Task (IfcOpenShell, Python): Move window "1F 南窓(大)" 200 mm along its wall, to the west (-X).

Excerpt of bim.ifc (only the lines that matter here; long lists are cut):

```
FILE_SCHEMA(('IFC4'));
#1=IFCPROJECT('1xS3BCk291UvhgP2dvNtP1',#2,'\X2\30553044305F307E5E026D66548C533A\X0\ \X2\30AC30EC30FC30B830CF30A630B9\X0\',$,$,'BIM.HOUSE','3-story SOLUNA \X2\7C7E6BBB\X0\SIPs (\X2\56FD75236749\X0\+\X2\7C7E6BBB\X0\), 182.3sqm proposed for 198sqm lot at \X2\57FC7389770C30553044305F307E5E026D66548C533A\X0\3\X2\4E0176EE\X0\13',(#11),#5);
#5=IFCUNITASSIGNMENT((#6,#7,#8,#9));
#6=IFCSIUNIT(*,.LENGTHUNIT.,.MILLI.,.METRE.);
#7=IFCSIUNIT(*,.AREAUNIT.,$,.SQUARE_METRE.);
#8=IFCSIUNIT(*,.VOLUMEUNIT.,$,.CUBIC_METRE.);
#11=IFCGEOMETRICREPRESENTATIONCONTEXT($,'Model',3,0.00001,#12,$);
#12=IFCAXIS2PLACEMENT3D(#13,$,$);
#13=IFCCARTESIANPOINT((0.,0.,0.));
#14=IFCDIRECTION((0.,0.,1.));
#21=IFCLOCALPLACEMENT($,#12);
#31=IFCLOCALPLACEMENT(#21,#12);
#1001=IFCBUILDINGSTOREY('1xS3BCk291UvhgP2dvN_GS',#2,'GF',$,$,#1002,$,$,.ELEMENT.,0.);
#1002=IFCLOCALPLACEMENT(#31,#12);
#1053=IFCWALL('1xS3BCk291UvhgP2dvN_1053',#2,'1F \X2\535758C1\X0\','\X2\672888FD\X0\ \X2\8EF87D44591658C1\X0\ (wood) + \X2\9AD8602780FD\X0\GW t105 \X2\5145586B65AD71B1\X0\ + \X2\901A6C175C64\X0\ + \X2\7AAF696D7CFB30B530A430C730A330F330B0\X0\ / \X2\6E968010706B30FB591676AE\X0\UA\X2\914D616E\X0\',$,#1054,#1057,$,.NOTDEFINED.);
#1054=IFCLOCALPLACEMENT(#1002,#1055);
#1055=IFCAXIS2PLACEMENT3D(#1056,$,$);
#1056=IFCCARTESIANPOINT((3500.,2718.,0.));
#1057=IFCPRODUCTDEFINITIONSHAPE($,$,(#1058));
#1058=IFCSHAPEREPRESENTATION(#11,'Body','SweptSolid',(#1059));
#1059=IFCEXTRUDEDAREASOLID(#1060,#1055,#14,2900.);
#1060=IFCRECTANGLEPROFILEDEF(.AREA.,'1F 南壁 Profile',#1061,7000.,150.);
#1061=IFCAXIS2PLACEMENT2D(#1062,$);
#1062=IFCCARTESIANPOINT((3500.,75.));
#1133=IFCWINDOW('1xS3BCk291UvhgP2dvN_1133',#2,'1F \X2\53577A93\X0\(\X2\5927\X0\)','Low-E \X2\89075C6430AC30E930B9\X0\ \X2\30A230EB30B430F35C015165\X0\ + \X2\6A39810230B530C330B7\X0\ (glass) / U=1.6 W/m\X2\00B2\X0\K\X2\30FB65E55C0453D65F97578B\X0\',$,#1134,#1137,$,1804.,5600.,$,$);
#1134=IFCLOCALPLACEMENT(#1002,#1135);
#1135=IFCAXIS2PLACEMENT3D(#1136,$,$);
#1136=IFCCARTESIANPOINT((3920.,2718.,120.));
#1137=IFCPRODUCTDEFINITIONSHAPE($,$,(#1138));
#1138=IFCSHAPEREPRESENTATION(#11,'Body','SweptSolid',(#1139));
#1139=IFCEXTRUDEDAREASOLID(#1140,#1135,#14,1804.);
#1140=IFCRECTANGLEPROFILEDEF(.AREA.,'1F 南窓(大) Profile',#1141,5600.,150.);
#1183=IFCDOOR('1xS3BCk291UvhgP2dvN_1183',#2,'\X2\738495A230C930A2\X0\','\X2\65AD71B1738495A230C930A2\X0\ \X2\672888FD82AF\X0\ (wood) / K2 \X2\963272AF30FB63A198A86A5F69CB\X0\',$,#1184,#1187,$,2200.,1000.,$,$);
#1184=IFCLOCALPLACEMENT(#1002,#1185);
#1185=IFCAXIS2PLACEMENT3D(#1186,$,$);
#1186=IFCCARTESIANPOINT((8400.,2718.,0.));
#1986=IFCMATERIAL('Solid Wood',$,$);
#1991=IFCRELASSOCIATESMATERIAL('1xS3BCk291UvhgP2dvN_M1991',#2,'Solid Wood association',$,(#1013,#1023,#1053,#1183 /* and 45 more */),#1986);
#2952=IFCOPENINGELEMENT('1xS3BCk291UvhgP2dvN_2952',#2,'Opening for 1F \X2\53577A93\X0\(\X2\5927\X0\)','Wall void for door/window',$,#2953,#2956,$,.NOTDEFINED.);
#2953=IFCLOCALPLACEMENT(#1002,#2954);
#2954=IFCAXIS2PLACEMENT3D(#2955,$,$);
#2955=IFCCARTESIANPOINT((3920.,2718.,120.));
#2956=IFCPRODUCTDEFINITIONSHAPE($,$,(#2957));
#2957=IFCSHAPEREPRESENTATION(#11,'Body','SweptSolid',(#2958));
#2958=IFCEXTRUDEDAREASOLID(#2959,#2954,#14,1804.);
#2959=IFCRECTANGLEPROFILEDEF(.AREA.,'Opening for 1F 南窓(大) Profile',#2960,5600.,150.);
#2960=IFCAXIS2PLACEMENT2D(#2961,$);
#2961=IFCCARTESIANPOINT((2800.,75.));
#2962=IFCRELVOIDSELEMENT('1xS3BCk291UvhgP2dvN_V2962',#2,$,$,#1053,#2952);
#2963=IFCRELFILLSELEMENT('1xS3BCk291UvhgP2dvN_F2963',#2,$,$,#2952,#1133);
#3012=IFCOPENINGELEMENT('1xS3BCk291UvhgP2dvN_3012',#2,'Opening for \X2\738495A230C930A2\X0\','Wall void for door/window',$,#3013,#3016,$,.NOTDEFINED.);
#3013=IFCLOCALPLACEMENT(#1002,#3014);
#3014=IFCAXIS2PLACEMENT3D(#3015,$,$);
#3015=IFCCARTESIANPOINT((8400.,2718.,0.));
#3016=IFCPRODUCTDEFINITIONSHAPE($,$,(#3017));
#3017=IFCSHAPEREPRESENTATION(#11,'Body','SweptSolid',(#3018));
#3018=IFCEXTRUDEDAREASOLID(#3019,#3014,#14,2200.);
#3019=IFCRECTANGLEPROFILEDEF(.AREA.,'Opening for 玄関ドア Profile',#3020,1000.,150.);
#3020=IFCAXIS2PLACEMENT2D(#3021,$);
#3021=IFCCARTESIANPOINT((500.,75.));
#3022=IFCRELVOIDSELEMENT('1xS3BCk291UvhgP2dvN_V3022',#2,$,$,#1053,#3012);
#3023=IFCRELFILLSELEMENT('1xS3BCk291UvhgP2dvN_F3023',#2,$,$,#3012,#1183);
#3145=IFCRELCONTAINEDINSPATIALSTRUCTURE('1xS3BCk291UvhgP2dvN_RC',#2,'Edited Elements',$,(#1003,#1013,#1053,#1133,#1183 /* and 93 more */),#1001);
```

```python
import ifcopenshell
import ifcopenshell.api.geometry
import ifcopenshell.util.placement

model = ifcopenshell.open("bim.ifc")

window = model.by_guid("1xS3BCk291UvhgP2dvN_1133")
opening = window.FillsVoids[0].RelatingOpeningElement
wall = opening.VoidsElements[0].RelatingBuildingElement

wall_matrix = ifcopenshell.util.placement.get_local_placement(wall.ObjectPlacement)
shift = wall_matrix[:3, 0] * -200.0
before = ifcopenshell.util.placement.get_local_placement(window.ObjectPlacement)[:3, 3].copy()

# The window is not placed relative to its opening, so move both.
for product in (opening, window):
    matrix = ifcopenshell.util.placement.get_local_placement(product.ObjectPlacement)
    matrix[:3, 3] += shift
    ifcopenshell.api.geometry.edit_object_placement(model, product=product, matrix=matrix, is_si=False)

after = ifcopenshell.util.placement.get_local_placement(window.ObjectPlacement)[:3, 3]
print("window moved by", (after - before).round(3) + 0.0)

model.write("bim_edited.ifc")
```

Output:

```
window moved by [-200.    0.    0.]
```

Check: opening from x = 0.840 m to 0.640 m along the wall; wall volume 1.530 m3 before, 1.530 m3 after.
